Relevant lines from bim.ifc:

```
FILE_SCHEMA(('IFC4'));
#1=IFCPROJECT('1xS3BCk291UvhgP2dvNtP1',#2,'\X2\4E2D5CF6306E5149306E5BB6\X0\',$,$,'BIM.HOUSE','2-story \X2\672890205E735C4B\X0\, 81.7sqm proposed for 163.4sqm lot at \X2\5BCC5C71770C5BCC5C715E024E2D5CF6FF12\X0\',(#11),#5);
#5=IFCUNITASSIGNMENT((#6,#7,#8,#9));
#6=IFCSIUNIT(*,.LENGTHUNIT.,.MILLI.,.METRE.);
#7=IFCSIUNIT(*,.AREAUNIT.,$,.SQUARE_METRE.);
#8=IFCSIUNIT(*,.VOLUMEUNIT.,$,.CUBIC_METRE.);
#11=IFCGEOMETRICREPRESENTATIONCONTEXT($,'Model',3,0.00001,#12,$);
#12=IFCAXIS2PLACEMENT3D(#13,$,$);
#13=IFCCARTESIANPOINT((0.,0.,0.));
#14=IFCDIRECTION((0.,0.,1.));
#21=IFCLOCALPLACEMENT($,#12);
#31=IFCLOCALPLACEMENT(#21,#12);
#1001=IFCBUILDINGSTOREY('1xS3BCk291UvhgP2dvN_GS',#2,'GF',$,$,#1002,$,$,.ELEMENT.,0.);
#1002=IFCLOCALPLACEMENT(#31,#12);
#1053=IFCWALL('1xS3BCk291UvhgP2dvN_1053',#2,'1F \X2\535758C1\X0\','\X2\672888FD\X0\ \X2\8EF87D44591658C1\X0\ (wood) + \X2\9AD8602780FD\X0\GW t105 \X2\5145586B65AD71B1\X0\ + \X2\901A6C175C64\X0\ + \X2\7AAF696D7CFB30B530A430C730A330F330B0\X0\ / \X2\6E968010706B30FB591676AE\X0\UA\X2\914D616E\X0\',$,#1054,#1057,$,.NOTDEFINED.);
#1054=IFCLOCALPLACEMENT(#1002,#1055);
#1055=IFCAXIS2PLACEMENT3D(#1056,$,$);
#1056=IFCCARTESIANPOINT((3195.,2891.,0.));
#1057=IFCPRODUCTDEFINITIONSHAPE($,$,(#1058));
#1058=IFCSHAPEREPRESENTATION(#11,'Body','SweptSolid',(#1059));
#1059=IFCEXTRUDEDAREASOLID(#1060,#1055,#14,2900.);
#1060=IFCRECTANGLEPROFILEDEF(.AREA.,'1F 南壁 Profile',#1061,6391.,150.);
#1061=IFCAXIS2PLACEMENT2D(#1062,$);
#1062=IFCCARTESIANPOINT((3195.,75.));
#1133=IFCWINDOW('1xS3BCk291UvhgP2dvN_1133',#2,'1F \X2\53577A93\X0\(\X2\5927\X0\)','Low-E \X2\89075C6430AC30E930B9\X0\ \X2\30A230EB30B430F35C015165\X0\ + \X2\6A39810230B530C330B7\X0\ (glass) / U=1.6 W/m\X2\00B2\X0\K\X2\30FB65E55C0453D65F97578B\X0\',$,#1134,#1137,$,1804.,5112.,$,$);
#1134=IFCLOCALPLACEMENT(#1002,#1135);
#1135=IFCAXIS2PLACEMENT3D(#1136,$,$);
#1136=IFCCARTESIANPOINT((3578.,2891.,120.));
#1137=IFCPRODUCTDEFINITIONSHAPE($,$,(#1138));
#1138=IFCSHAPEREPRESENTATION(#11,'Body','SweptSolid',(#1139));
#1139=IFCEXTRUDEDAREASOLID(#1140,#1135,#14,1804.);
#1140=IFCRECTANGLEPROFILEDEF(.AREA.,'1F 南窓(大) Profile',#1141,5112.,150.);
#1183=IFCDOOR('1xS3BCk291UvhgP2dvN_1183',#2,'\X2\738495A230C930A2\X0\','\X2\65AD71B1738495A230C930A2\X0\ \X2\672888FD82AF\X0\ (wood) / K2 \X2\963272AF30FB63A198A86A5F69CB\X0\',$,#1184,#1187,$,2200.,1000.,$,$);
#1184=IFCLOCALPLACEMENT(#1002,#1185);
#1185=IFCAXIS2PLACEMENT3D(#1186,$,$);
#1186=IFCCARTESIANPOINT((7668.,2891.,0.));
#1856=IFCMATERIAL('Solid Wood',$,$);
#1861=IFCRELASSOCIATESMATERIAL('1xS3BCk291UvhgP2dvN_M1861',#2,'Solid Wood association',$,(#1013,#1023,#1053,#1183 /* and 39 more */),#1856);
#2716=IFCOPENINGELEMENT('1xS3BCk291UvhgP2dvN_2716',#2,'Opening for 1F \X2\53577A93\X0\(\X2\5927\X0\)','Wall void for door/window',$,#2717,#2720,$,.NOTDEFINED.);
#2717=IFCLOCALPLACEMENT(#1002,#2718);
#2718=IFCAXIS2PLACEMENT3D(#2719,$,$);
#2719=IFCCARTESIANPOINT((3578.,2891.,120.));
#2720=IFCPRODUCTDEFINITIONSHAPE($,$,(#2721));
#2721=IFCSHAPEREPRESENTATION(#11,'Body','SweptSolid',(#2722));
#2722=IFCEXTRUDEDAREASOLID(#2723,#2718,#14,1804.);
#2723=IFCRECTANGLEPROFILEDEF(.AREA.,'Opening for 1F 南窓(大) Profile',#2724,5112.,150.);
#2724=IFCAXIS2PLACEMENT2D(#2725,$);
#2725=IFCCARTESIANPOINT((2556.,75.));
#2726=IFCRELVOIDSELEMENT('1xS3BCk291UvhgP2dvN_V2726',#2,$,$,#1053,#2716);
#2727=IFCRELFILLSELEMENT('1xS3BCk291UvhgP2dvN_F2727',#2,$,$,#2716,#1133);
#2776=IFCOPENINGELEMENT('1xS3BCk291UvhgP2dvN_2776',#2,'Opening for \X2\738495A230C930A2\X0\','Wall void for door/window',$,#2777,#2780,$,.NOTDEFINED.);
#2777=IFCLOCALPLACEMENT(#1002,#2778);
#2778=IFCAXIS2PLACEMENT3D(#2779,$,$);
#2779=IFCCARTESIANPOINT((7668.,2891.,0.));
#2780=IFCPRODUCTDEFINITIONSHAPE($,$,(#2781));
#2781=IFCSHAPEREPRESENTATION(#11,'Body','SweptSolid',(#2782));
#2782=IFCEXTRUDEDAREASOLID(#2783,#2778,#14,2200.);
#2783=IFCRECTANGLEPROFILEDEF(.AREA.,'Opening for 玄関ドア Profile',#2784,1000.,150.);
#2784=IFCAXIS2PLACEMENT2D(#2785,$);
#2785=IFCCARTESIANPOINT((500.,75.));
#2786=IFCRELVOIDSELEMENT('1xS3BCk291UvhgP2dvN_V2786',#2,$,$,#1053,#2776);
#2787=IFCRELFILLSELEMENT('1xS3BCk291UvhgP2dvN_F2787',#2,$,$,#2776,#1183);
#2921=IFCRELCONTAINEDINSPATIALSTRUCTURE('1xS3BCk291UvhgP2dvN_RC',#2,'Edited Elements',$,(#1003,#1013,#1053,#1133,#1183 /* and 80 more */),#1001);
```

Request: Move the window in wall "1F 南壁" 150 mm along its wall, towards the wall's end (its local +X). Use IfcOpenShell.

```python
import ifcopenshell
import ifcopenshell.api.geometry
import ifcopenshell.util.placement
import ifcopenshell.util.unit

model = ifcopenshell.open("bim.ifc")
unit_scale = ifcopenshell.util.unit.calculate_unit_scale(model)

window = model.by_id(1133)
opening = window.FillsVoids[0].RelatingOpeningElement
wall = opening.VoidsElements[0].RelatingBuildingElement

wall_matrix = ifcopenshell.util.placement.get_local_placement(wall.ObjectPlacement)
shift = wall_matrix[:3, 0] * 0.15 / unit_scale
before = ifcopenshell.util.placement.get_local_placement(window.ObjectPlacement)[:3, 3].copy()

# The window is not placed relative to its opening, so move both.
for product in (opening, window):
    matrix = ifcopenshell.util.placement.get_local_placement(product.ObjectPlacement)
    matrix[:3, 3] += shift
    ifcopenshell.api.geometry.edit_object_placement(model, product=product, matrix=matrix, is_si=False)

after = ifcopenshell.util.placement.get_local_placement(window.ObjectPlacement)[:3, 3]
print("window moved by", (after - before).round(3) + 0.0)

model.write("bim-out.ifc")
```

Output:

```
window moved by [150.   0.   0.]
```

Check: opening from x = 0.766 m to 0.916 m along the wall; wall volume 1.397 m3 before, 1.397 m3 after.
